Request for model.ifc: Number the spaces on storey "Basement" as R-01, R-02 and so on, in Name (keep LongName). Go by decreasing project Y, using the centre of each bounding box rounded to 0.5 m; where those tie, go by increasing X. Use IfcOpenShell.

First a look at what the model holds.

```python
import ifcopenshell
import ifcopenshell.util.element
import ifcopenshell.util.placement

model = ifcopenshell.open("model.ifc")
print(model.schema)
storey = next(s for s in model.by_type("IfcBuildingStorey") if s.Name == "Basement")
spaces = [e for e in ifcopenshell.util.element.get_decomposition(storey) if e.is_a("IfcSpace")]
for e in sorted(spaces, key=lambda e: e.id()):
    origin = ifcopenshell.util.placement.get_local_placement(e.ObjectPlacement)[:3, 3]
    print(e.id(), e.Name, e.LongName, origin.round(2) + 0.0, sep=" | ")
```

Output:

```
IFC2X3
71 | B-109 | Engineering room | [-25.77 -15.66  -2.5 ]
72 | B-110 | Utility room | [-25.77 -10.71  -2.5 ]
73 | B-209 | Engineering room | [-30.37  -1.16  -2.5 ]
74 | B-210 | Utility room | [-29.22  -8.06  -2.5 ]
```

```python
import ifcopenshell
import ifcopenshell.geom
import ifcopenshell.util.element
import ifcopenshell.util.shape

model = ifcopenshell.open("model.ifc")
settings = ifcopenshell.geom.settings()
settings.set("use-world-coords", True)


def centre(element):
    shape = ifcopenshell.geom.create_shape(settings, element)
    return ifcopenshell.util.shape.get_bbox_centroid(shape.geometry)


storey = next(s for s in model.by_type("IfcBuildingStorey") if s.Name == "Basement")
spaces = [e for e in ifcopenshell.util.element.get_decomposition(storey) if e.is_a("IfcSpace")]

# Insertion points can sit at a corner or the storey origin, so sort by the geometry (in metres).
centres = {e: centre(e) for e in spaces}
spaces.sort(key=lambda e: (-round(centres[e][1] / 0.5), centres[e][0]))

for i, e in enumerate(spaces, start=1):
    number = f"R-{i:02d}"
    e.Name = number
    print(e.id(), number)

model.write("model_v2.ifc")
```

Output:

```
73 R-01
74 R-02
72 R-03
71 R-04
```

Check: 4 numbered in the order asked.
